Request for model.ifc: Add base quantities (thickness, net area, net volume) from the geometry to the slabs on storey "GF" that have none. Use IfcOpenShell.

First a look at what the model holds.

```python
import ifcopenshell
import ifcopenshell.util.element
import ifcopenshell.util.unit

model = ifcopenshell.open("model.ifc")
print(model.schema)
for unit_type in ("LENGTHUNIT", "AREAUNIT", "VOLUMEUNIT"):
    print(unit_type, ifcopenshell.util.unit.calculate_unit_scale(model, unit_type))
storey = next(s for s in model.by_type("IfcBuildingStorey") if s.Name == "GF")
slabs = [e for e in ifcopenshell.util.element.get_decomposition(storey) if e.is_a("IfcSlab")]
for e in sorted(slabs, key=lambda e: e.id()):
    print(e.id(), e.is_a(), e.Name, list(ifcopenshell.util.element.get_psets(e, qtos_only=True)), sep=" | ")
```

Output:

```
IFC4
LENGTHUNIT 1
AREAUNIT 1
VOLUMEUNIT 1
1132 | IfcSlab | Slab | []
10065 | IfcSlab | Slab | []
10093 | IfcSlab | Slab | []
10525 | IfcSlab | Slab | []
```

```python
import ifcopenshell
import ifcopenshell.api.pset
import ifcopenshell.geom
import ifcopenshell.util.element
import ifcopenshell.util.shape
import ifcopenshell.util.unit

model = ifcopenshell.open("model.ifc")
unit_scale = ifcopenshell.util.unit.calculate_unit_scale(model)
area_scale = ifcopenshell.util.unit.calculate_unit_scale(model, "AREAUNIT")
volume_scale = ifcopenshell.util.unit.calculate_unit_scale(model, "VOLUMEUNIT")
settings = ifcopenshell.geom.settings()

storey = next(s for s in model.by_type("IfcBuildingStorey") if s.Name == "GF")
slabs = [e for e in ifcopenshell.util.element.get_decomposition(storey) if e.is_a("IfcSlab")]

for e in sorted(slabs, key=lambda e: e.id()):
    if ifcopenshell.util.element.get_psets(e, qtos_only=True, should_inherit=False):
        continue
    # Geometry comes back in metres, in the element's own axes.
    shape = ifcopenshell.geom.create_shape(settings, e)
    values = {
        "Width": ifcopenshell.util.shape.get_z(shape.geometry) / unit_scale,
        "NetArea": ifcopenshell.util.shape.get_footprint_area(shape.geometry) / area_scale,
        "NetVolume": ifcopenshell.util.shape.get_volume(shape.geometry) / volume_scale,
    }
    qto = ifcopenshell.api.pset.add_qto(model, product=e, name="Qto_SlabBaseQuantities")
    ifcopenshell.api.pset.edit_qto(model, qto=qto, properties=values)
    print(e.id(), {k: round(v, 3) for k, v in values.items()})

model.write("model_updated.ifc")
```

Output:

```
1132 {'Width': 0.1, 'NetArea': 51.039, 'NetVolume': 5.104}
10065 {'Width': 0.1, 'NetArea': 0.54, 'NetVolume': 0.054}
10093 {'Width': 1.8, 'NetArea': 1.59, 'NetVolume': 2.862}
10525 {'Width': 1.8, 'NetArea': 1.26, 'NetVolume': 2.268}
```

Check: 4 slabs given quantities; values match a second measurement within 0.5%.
